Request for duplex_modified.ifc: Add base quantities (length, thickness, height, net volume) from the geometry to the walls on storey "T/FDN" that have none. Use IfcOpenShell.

First a look at what the model holds.

```python
import ifcopenshell
import ifcopenshell.util.element
import ifcopenshell.util.unit

model = ifcopenshell.open("duplex_modified.ifc")
print(model.schema)
for unit_type in ("LENGTHUNIT", "AREAUNIT", "VOLUMEUNIT"):
    print(unit_type, ifcopenshell.util.unit.calculate_unit_scale(model, unit_type))
storey = next(s for s in model.by_type("IfcBuildingStorey") if s.Name == "T/FDN")
walls = [e for e in ifcopenshell.util.element.get_decomposition(storey) if e.is_a("IfcWall")]
for e in sorted(walls, key=lambda e: e.id()):
    print(e.id(), e.is_a(), e.Name, list(ifcopenshell.util.element.get_psets(e, qtos_only=True)), sep=" | ")
```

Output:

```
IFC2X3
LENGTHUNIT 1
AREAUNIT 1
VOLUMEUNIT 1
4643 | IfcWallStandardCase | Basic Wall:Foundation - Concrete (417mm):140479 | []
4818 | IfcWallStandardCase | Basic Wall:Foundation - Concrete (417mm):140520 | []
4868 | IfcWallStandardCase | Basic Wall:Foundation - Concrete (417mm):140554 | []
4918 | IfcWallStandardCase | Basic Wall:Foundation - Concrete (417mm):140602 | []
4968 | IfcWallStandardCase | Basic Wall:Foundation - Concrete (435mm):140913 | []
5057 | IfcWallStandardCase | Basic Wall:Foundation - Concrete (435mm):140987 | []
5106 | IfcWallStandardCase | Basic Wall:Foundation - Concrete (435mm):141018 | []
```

```python
import ifcopenshell
import ifcopenshell.api.pset
import ifcopenshell.geom
import ifcopenshell.util.element
import ifcopenshell.util.shape
import ifcopenshell.util.unit

model = ifcopenshell.open("duplex_modified.ifc")
unit_scale = ifcopenshell.util.unit.calculate_unit_scale(model)
volume_scale = ifcopenshell.util.unit.calculate_unit_scale(model, "VOLUMEUNIT")
settings = ifcopenshell.geom.settings()

storey = next(s for s in model.by_type("IfcBuildingStorey") if s.Name == "T/FDN")
walls = [e for e in ifcopenshell.util.element.get_decomposition(storey) if e.is_a("IfcWall")]

for e in sorted(walls, key=lambda e: e.id()):
    if ifcopenshell.util.element.get_psets(e, qtos_only=True, should_inherit=False):
        continue
    # Geometry comes back in metres, in the element's own axes.
    shape = ifcopenshell.geom.create_shape(settings, e)
    values = {
        "Length": ifcopenshell.util.shape.get_x(shape.geometry) / unit_scale,
        "Width": ifcopenshell.util.shape.get_y(shape.geometry) / unit_scale,
        "Height": ifcopenshell.util.shape.get_z(shape.geometry) / unit_scale,
        "NetVolume": ifcopenshell.util.shape.get_volume(shape.geometry) / volume_scale,
    }
    qto = ifcopenshell.api.pset.add_qto(model, product=e, name="BaseQuantities")
    ifcopenshell.api.pset.edit_qto(model, qto=qto, properties=values)
    print(e.id(), {k: round(v, 3) for k, v in values.items()})

model.write("duplex_modified_rev.ifc")
```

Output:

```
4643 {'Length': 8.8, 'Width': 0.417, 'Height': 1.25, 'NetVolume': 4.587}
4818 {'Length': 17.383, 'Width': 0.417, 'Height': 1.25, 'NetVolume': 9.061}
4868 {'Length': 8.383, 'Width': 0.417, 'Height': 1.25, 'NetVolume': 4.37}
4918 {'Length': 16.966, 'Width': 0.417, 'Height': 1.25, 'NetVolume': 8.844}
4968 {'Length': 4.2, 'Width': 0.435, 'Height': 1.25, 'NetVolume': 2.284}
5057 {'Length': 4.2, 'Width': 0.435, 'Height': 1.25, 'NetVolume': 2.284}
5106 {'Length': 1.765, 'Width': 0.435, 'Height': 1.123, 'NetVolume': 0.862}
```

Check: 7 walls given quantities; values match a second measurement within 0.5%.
